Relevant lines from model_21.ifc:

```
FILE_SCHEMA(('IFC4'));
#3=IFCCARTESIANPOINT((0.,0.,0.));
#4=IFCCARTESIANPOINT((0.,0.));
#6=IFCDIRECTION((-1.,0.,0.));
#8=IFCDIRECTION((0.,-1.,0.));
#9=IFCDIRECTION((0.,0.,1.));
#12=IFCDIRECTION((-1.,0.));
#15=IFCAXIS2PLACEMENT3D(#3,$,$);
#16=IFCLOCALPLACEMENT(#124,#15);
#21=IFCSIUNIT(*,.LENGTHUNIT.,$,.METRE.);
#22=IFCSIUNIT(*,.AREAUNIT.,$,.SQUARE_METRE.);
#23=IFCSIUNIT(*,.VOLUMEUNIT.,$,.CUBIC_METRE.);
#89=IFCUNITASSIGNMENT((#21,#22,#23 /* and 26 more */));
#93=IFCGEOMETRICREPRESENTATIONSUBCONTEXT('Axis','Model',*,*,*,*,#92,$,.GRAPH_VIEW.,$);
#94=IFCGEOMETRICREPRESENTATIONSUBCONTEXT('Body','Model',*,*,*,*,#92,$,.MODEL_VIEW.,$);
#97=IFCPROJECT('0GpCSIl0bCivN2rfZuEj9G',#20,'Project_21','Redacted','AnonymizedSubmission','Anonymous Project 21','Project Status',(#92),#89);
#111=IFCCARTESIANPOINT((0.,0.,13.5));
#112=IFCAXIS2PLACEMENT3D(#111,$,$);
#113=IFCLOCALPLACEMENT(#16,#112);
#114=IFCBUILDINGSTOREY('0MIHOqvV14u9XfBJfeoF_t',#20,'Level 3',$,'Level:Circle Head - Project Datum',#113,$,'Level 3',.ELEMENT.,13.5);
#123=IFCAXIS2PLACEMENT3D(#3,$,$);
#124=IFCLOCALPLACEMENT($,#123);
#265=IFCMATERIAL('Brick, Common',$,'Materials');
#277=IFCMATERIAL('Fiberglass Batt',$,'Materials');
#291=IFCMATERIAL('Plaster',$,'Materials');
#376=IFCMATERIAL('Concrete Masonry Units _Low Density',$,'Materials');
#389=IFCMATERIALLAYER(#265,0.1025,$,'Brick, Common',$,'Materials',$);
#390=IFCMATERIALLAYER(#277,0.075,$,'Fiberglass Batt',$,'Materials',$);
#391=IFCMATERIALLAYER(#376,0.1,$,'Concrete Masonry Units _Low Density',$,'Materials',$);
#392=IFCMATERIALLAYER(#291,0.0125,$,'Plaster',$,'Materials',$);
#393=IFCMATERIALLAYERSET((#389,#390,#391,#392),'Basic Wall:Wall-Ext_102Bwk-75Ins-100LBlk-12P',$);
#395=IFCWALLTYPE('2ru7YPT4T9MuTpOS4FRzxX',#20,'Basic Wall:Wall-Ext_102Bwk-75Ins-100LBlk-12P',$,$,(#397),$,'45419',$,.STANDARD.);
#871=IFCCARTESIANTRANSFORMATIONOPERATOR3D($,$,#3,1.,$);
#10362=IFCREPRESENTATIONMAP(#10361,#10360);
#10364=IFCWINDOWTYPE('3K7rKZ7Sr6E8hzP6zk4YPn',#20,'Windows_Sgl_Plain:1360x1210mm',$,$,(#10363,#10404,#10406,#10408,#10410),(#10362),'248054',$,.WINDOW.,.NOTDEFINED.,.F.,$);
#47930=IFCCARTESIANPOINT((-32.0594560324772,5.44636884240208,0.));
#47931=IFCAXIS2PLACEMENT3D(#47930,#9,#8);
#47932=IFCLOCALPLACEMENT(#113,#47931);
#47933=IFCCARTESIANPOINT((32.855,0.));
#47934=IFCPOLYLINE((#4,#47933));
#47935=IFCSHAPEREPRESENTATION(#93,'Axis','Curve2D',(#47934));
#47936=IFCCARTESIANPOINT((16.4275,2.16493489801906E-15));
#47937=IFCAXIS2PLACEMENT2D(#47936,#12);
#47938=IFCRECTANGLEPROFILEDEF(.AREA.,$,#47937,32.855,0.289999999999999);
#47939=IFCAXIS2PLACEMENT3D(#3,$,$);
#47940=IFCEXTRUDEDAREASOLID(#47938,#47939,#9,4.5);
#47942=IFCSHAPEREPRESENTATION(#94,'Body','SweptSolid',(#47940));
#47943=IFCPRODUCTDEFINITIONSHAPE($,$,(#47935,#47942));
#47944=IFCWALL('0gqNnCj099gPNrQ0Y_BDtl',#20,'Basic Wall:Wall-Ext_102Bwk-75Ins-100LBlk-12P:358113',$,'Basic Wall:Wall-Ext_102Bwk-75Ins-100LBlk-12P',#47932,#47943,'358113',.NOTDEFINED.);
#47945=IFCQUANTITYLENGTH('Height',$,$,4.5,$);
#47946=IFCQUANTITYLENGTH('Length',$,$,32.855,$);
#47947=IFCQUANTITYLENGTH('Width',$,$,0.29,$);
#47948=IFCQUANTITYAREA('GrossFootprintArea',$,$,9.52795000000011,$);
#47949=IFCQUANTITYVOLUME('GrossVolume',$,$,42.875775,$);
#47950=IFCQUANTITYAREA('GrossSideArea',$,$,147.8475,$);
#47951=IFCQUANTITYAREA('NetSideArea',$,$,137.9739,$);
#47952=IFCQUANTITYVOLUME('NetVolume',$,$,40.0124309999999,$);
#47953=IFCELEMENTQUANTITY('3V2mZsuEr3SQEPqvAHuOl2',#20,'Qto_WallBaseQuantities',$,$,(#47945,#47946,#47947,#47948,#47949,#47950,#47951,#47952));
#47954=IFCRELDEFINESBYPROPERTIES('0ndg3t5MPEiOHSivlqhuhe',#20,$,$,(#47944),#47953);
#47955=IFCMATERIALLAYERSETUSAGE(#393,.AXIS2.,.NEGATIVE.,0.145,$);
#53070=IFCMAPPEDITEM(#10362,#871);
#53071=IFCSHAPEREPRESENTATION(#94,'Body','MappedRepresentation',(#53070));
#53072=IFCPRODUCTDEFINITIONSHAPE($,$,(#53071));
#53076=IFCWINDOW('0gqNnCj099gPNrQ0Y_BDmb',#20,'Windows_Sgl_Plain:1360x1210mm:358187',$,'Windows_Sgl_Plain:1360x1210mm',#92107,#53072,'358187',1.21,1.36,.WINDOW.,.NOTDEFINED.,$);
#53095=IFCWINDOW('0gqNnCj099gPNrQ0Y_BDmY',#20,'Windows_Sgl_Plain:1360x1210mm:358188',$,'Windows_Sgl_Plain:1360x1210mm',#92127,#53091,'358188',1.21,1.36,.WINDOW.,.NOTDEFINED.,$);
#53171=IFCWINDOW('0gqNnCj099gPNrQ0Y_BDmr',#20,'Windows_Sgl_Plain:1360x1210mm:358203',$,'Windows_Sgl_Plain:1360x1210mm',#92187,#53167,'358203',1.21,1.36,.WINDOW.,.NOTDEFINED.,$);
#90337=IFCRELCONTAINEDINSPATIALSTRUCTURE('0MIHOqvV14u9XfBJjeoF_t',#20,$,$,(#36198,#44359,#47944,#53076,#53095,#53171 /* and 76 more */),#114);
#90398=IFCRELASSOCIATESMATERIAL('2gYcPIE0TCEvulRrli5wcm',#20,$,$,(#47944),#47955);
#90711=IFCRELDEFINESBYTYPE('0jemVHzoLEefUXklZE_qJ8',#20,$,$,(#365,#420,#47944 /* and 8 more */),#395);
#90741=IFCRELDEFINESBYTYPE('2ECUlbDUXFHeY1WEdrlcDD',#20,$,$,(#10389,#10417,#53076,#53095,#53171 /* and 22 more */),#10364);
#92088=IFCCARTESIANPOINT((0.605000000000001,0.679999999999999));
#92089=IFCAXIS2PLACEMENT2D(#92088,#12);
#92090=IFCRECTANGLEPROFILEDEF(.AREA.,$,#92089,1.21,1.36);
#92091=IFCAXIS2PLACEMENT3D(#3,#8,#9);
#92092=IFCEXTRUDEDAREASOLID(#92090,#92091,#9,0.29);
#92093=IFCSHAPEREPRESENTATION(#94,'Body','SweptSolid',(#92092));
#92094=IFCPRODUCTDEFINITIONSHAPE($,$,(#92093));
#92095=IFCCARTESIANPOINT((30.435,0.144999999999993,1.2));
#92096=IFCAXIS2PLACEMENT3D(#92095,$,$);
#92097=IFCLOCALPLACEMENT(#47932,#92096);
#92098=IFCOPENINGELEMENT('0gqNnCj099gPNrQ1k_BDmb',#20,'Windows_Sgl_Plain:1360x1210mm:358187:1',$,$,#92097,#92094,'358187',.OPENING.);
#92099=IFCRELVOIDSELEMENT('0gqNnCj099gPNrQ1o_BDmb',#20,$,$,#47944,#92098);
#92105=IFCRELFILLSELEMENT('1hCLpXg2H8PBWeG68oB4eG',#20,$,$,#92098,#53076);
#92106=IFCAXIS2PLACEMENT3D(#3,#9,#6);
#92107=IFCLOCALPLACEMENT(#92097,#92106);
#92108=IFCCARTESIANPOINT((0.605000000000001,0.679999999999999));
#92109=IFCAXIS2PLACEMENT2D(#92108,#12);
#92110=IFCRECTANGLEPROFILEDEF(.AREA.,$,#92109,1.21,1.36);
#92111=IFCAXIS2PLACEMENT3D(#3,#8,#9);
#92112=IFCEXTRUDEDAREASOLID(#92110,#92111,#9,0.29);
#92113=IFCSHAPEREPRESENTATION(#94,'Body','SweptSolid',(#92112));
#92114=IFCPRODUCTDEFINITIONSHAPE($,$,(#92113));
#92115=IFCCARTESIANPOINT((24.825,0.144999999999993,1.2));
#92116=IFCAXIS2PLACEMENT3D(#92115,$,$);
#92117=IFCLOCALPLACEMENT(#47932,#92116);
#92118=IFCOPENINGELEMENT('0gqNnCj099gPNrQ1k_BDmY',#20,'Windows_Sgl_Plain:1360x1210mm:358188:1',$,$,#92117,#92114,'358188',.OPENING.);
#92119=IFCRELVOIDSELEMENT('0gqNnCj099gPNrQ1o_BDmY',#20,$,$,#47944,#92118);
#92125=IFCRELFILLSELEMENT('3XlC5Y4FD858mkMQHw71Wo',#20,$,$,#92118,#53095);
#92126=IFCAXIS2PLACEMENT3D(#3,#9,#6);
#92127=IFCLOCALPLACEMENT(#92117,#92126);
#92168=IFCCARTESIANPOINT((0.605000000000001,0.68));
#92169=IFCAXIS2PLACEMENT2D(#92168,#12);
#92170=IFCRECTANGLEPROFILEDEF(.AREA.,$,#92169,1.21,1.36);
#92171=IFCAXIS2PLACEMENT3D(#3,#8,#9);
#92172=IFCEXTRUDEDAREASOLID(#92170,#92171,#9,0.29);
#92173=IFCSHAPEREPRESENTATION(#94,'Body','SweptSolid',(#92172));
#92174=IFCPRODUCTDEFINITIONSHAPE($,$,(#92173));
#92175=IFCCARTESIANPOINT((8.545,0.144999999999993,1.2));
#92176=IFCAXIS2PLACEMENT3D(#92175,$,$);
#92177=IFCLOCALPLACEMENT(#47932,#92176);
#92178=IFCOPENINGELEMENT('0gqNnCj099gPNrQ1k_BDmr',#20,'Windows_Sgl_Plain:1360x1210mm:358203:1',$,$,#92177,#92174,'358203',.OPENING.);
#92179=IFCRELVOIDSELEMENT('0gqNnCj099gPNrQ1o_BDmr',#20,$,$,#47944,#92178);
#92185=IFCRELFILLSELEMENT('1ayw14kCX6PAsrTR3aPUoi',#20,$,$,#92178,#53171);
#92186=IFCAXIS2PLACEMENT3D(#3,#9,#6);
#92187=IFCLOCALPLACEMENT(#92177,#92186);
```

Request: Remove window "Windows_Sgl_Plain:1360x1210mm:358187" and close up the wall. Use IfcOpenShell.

```python
import ifcopenshell
import ifcopenshell.api.feature
import ifcopenshell.api.pset
import ifcopenshell.api.root
import ifcopenshell.geom
import ifcopenshell.util.element
import ifcopenshell.util.shape
import ifcopenshell.util.unit

model = ifcopenshell.open("model_21.ifc")
area_scale = ifcopenshell.util.unit.calculate_unit_scale(model, "AREAUNIT")
volume_scale = ifcopenshell.util.unit.calculate_unit_scale(model, "VOLUMEUNIT")
settings = ifcopenshell.geom.settings()


def volume(element):
    """Net volume in cubic metres, openings subtracted."""
    shape = ifcopenshell.geom.create_shape(settings, element)
    return ifcopenshell.util.shape.get_volume(shape.geometry)


window = model.by_guid("0gqNnCj099gPNrQ0Y_BDmb")
opening = window.FillsVoids[0].RelatingOpeningElement
wall = opening.VoidsElements[0].RelatingBuildingElement
before = volume(wall)

ifcopenshell.api.root.remove_product(model, product=window)
ifcopenshell.api.feature.remove_feature(model, feature=opening)

after = volume(wall)
thickness = 0.29  # wall thickness in metres

# Update the wall's stored quantities.
qto = model.by_id(ifcopenshell.util.element.get_pset(wall, "Qto_WallBaseQuantities", should_inherit=False)["id"])
ifcopenshell.api.pset.edit_qto(model, qto=qto, properties={
    "NetSideArea": after / thickness / area_scale,
    "NetVolume": after / volume_scale,
})

print(f"wall volume {before:.3f} -> {after:.3f} m3")

model.write("model_21-out.ifc")
```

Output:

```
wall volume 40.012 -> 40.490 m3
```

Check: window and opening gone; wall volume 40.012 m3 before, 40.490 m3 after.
